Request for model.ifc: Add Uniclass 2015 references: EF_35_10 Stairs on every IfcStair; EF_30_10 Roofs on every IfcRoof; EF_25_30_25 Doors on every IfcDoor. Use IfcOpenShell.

First a look at what the model holds.

```python
import ifcopenshell

model = ifcopenshell.open("model.ifc")
print(model.schema)
print("classifications:", [c.Name for c in model.by_type("IfcClassification")])
for ifc_class in ("IfcDoor", "IfcRoof", "IfcStair", "IfcWall", "IfcWindow"):
    print(ifc_class, len(model.by_type(ifc_class)))
```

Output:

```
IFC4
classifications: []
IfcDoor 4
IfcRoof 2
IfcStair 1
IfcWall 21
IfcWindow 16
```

```python
import ifcopenshell
import ifcopenshell.api.classification

model = ifcopenshell.open("model.ifc")

system = ifcopenshell.api.classification.add_classification(model, classification="Uniclass 2015")

codes = {
    "IfcStair": ("EF_35_10", "Stairs"),
    "IfcRoof": ("EF_30_10", "Roofs"),
    "IfcDoor": ("EF_25_30_25", "Doors"),
}
for ifc_class, (code, name) in codes.items():
    products = model.by_type(ifc_class)
    ifcopenshell.api.classification.add_reference(
        model, products=products, classification=system, identification=code, name=name
    )
    print(code, len(products))

model.write("model_v2.ifc")
```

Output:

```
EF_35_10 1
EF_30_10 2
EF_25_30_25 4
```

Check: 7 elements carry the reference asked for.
